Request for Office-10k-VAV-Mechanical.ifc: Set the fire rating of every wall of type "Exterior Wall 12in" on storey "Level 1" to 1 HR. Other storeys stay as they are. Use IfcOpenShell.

First a look at what the model holds.

```python
import ifcopenshell
import ifcopenshell.util.element

model = ifcopenshell.open("Office-10k-VAV-Mechanical.ifc")
print(model.schema)
storey = next(s for s in model.by_type("IfcBuildingStorey") if s.Name == "Level 1")
walls = [e for e in ifcopenshell.util.element.get_decomposition(storey) if e.is_a("IfcWall")]
seen = {}
for e in walls:
    element_type = ifcopenshell.util.element.get_type(e)
    key = (element_type.Name if element_type != e and element_type else None, ifcopenshell.util.element.get_pset(e, "Pset_WallCommon", "FireRating"))
    seen[key] = seen.get(key, 0) + 1
for (name, value), count in sorted(seen.items(), key=str):
    print(count, "x", name, "|", value)
```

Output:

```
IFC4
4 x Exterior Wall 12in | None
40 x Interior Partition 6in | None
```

```python
import ifcopenshell
import ifcopenshell.api.pset
import ifcopenshell.util.element

model = ifcopenshell.open("Office-10k-VAV-Mechanical.ifc")

storey = next(s for s in model.by_type("IfcBuildingStorey") if s.Name == "Level 1")
walls = [e for e in ifcopenshell.util.element.get_decomposition(storey) if e.is_a("IfcWall")]

count = 0
for e in walls:
    element_type = ifcopenshell.util.element.get_type(e)
    if element_type in (None, e) or element_type.Name != "Exterior Wall 12in":
        continue
    # add_pset returns the element's existing set when there is one.
    pset = ifcopenshell.api.pset.add_pset(model, product=e, name="Pset_WallCommon")
    ifcopenshell.api.pset.edit_pset(model, pset=pset, properties={"FireRating": "1 HR"})
    count += 1

print(count, "walls updated")

model.write("Office-10k-VAV-Mechanical_updated.ifc")
```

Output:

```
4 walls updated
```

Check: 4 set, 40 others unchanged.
